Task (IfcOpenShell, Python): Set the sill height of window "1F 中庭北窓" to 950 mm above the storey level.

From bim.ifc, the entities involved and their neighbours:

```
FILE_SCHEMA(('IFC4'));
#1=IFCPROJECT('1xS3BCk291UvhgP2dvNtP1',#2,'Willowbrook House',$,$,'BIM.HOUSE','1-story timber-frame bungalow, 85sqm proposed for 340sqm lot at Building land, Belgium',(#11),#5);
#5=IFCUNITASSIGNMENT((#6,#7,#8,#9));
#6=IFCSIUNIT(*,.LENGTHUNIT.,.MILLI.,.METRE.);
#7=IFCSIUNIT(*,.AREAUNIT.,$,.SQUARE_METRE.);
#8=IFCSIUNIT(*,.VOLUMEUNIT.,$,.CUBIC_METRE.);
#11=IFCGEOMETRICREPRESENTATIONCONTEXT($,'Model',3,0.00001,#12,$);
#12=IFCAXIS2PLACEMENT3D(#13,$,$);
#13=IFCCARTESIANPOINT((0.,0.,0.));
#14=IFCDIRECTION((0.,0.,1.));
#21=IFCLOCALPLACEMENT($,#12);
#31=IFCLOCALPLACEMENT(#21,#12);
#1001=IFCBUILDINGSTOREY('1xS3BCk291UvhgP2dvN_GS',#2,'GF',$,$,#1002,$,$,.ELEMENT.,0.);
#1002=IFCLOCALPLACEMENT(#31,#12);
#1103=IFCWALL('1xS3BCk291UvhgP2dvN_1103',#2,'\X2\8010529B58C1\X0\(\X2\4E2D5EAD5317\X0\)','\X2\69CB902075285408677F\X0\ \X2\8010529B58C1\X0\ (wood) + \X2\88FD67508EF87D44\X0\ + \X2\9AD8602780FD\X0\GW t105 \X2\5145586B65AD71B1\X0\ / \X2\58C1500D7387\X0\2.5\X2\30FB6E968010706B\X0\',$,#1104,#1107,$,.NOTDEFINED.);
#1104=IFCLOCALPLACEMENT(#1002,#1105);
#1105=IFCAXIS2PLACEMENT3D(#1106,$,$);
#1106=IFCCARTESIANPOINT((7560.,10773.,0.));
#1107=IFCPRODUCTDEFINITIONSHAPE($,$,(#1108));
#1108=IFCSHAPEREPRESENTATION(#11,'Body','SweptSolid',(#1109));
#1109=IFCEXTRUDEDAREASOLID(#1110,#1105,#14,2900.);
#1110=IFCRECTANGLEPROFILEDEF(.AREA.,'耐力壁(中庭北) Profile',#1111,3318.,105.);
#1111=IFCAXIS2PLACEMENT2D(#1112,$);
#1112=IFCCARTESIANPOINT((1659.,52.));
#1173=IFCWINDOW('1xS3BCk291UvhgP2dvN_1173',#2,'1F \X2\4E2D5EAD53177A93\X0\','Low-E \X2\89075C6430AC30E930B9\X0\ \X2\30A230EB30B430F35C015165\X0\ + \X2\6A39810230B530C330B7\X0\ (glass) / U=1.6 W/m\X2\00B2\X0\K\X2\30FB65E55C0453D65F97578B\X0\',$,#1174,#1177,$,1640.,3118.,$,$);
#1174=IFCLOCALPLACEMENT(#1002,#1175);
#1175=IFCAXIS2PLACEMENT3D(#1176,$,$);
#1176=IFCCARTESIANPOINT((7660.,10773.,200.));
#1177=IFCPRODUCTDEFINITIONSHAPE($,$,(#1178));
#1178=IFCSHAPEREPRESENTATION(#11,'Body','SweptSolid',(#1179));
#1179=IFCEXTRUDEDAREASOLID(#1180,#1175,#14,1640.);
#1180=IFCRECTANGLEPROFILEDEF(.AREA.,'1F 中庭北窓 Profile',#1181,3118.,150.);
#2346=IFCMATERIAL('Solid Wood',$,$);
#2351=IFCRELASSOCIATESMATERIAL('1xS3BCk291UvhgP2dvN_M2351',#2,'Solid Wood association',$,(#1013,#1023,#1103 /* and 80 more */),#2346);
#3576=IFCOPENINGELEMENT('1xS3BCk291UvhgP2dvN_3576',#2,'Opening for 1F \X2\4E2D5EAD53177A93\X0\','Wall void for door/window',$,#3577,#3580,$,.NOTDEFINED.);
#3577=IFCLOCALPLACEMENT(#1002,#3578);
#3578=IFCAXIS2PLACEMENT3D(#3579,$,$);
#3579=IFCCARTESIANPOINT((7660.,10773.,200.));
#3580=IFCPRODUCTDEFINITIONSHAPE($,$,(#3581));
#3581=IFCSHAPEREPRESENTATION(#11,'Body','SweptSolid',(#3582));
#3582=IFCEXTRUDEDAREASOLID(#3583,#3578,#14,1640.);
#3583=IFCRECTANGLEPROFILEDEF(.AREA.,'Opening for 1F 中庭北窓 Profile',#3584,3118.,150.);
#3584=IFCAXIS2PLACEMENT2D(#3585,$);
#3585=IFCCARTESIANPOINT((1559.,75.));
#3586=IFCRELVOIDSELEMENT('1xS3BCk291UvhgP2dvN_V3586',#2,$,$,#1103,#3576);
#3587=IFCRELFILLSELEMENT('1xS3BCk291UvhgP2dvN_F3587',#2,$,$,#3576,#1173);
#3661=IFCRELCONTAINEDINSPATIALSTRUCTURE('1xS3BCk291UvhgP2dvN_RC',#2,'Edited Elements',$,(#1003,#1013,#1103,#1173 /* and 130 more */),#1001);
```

```python
import numpy as np
import ifcopenshell
import ifcopenshell.api.geometry
import ifcopenshell.geom
import ifcopenshell.util.element
import ifcopenshell.util.placement
import ifcopenshell.util.shape
import ifcopenshell.util.unit

model = ifcopenshell.open("bim.ifc")
unit_scale = ifcopenshell.util.unit.calculate_unit_scale(model)

window = model.by_id(1173)
opening = window.FillsVoids[0].RelatingOpeningElement
storey = ifcopenshell.util.element.get_container(window, ifc_class="IfcBuildingStorey")
level = ifcopenshell.util.placement.get_local_placement(storey.ObjectPlacement)[2, 3]

# The opening's origin need not be at the sill, so measure its lowest point.
shape = ifcopenshell.geom.create_shape(ifcopenshell.geom.settings(), opening)
bottom = ifcopenshell.util.shape.get_shape_bottom_elevation(shape, shape.geometry) / unit_scale
dz = level + 950.0 - bottom

shift = np.array([0.0, 0.0, dz])
# The window is not placed relative to its opening, so move both.
for product in (opening, window):
    matrix = ifcopenshell.util.placement.get_local_placement(product.ObjectPlacement)
    matrix[:3, 3] += shift
    ifcopenshell.api.geometry.edit_object_placement(model, product=product, matrix=matrix, is_si=False)

print(f"moved by {dz * unit_scale:+.3f} m")

model.write("bim_v2.ifc")
```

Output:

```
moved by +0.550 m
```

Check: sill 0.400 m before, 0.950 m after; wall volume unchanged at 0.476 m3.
